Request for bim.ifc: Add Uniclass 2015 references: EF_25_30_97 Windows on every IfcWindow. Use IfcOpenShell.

First a look at what the model holds.

```python
import ifcopenshell

model = ifcopenshell.open("bim.ifc")
print(model.schema)
print("classifications:", [c.Name for c in model.by_type("IfcClassification")])
for ifc_class in ("IfcDoor", "IfcRoof", "IfcStair", "IfcWall", "IfcWindow"):
    print(ifc_class, len(model.by_type(ifc_class)))
```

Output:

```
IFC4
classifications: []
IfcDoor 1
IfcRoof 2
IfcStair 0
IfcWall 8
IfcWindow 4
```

```python
import ifcopenshell
import ifcopenshell.api.classification

model = ifcopenshell.open("bim.ifc")

system = ifcopenshell.api.classification.add_classification(model, classification="Uniclass 2015")

codes = {
    "IfcWindow": ("EF_25_30_97", "Windows"),
}
for ifc_class, (code, name) in codes.items():
    products = model.by_type(ifc_class)
    ifcopenshell.api.classification.add_reference(
        model, products=products, classification=system, identification=code, name=name
    )
    print(code, len(products))

model.write("bim_rev.ifc")
```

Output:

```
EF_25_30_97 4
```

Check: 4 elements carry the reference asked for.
